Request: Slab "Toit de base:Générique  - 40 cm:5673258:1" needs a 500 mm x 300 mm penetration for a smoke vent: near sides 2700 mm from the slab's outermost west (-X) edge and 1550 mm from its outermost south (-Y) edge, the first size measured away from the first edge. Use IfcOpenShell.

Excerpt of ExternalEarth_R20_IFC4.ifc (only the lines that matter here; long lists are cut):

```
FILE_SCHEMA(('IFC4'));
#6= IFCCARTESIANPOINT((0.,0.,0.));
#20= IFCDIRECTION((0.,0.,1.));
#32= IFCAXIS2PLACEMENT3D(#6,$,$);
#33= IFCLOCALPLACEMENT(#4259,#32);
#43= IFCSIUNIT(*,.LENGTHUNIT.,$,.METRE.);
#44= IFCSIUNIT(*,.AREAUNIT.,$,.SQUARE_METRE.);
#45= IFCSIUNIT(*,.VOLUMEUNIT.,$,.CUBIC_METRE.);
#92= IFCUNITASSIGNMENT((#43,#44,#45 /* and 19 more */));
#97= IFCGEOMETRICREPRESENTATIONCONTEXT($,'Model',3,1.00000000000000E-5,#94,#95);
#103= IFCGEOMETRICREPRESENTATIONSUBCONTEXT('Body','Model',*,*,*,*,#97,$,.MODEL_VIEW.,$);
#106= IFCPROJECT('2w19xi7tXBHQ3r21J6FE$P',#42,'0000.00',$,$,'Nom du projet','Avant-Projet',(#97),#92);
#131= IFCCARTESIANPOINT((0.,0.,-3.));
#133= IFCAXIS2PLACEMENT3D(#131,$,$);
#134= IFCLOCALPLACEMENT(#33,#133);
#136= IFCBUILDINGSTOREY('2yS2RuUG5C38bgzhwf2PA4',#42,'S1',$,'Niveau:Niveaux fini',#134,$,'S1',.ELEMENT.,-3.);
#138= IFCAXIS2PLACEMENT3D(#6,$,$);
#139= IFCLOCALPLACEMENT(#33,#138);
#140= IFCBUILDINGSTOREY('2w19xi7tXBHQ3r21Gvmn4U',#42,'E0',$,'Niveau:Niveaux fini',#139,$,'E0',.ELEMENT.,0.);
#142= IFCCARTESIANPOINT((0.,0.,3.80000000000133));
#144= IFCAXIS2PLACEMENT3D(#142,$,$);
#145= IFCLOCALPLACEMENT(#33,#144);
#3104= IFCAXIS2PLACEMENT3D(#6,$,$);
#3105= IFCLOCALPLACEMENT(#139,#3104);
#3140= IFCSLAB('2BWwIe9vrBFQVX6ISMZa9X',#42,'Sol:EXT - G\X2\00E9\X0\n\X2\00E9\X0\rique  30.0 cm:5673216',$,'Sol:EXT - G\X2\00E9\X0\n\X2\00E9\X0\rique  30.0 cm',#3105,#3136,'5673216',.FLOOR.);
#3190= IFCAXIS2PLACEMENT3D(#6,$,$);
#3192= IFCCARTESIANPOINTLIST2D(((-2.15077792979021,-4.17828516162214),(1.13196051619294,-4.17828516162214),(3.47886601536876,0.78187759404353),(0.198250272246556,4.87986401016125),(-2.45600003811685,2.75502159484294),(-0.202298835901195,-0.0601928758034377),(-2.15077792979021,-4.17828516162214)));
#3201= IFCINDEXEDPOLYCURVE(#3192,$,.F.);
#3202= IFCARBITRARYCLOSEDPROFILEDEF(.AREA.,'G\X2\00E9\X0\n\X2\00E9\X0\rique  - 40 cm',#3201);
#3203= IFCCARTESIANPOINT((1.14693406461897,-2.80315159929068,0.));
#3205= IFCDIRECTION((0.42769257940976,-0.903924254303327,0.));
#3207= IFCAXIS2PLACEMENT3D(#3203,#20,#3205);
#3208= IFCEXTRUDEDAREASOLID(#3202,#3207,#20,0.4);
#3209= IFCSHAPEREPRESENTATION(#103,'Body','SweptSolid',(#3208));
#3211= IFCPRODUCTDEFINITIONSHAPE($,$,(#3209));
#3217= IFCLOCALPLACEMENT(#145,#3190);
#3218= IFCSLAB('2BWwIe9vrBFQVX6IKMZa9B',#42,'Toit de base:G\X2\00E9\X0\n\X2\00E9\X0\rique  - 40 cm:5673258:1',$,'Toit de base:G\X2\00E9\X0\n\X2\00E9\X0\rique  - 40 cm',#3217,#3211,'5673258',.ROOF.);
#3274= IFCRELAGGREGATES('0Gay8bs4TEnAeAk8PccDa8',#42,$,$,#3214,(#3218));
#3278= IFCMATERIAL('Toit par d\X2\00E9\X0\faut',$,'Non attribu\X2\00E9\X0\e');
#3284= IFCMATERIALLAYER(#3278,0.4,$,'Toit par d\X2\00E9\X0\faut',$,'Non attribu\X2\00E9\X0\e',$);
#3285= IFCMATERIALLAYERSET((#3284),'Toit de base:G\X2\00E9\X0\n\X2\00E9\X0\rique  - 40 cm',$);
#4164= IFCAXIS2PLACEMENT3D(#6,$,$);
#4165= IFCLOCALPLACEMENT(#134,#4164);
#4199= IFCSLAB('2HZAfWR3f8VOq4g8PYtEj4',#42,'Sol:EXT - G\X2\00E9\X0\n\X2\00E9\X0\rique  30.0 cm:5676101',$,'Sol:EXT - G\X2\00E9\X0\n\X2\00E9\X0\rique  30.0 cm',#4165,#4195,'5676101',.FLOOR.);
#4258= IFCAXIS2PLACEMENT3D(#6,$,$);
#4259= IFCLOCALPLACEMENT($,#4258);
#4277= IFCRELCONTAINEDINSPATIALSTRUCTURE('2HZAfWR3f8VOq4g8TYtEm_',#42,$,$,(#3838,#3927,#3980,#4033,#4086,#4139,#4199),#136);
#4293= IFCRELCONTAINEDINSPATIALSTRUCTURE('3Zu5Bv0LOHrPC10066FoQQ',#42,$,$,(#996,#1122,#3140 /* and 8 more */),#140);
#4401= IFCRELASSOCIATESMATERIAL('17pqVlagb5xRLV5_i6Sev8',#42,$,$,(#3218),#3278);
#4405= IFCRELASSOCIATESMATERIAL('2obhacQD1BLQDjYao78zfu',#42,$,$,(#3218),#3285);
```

```python
import numpy as np
import ifcopenshell
import ifcopenshell.api.feature
import ifcopenshell.api.geometry
import ifcopenshell.api.root
import ifcopenshell.geom
import ifcopenshell.util.placement
import ifcopenshell.util.representation
import ifcopenshell.util.shape
import ifcopenshell.util.unit

model = ifcopenshell.open("ExternalEarth_R20_IFC4.ifc")
unit_scale = ifcopenshell.util.unit.calculate_unit_scale(model)
settings = ifcopenshell.geom.settings()


def volume(element):
    """Net volume in cubic metres, openings subtracted."""
    shape = ifcopenshell.geom.create_shape(settings, element)
    return ifcopenshell.util.shape.get_volume(shape.geometry)


slab = model.by_id(3218)
before = volume(slab)

# Extent in the slab's own axes, in metres. The edges named are its -X and -Y sides.
slab_shape = ifcopenshell.geom.create_shape(settings, slab)
vertices = ifcopenshell.util.shape.get_vertices(slab_shape.geometry)
x_min, y_min, bottom = vertices.min(axis=0)
top = vertices[:, 2].max()

opening = ifcopenshell.api.root.create_entity(model, ifc_class="IfcOpeningElement", name="Smoke vent opening", predefined_type="OPENING")
context = ifcopenshell.util.representation.get_context(model, "Model", "Body", "MODEL_VIEW")
width, depth = 0.5, 0.3
outline = [(0.0, 0.0), (width, 0.0), (width, depth), (0.0, depth), (0.0, 0.0)]
# Overshoot both faces by 50 mm so the cut is clean.
shape = ifcopenshell.api.geometry.add_slab_representation(
    model, context=context, depth=top - bottom + 0.1, polyline=outline
)
ifcopenshell.api.geometry.assign_representation(model, product=opening, representation=shape)

matrix = ifcopenshell.util.placement.get_local_placement(slab.ObjectPlacement)
matrix[:, 3] = matrix @ np.append(np.array([x_min + 2.7, y_min + 1.55, bottom - 0.05]) / unit_scale, 1.0)
ifcopenshell.api.geometry.edit_object_placement(model, product=opening, matrix=matrix, is_si=False)
ifcopenshell.api.feature.add_feature(model, feature=opening, element=slab)

after = volume(slab)

print(f"slab volume {before:.3f} -> {after:.3f} m3")

model.write("ExternalEarth_R20_IFC4_edited.ifc")
```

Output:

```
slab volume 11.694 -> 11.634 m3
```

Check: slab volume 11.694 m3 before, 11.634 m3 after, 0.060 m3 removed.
